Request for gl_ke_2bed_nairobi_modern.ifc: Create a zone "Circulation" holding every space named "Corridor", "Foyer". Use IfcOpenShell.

First a look at what the model holds.

```python
import ifcopenshell

model = ifcopenshell.open("gl_ke_2bed_nairobi_modern.ifc")
print(model.schema)
seen = {}
for space in model.by_type("IfcSpace"):
    seen[space.LongName] = seen.get(space.LongName, 0) + 1
for name, count in sorted(seen.items(), key=str):
    print(count, "x", name)
print("zones:", [z.Name for z in model.by_type("IfcZone")][:20])
```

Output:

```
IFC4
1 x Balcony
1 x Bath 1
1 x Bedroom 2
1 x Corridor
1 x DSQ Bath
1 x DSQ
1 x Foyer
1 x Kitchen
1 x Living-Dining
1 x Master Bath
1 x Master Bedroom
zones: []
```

```python
import ifcopenshell
import ifcopenshell.api.group
import ifcopenshell.api.root

model = ifcopenshell.open("gl_ke_2bed_nairobi_modern.ifc")

names = {"Corridor", "Foyer"}
spaces = [s for s in model.by_type("IfcSpace") if s.LongName in names]

zone = ifcopenshell.api.root.create_entity(model, ifc_class="IfcZone", name="Circulation")
ifcopenshell.api.group.assign_group(model, products=spaces, group=zone)
print(len(spaces), "spaces in", zone.Name)

model.write("gl_ke_2bed_nairobi_modern_v2.ifc")
```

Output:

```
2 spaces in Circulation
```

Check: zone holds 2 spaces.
